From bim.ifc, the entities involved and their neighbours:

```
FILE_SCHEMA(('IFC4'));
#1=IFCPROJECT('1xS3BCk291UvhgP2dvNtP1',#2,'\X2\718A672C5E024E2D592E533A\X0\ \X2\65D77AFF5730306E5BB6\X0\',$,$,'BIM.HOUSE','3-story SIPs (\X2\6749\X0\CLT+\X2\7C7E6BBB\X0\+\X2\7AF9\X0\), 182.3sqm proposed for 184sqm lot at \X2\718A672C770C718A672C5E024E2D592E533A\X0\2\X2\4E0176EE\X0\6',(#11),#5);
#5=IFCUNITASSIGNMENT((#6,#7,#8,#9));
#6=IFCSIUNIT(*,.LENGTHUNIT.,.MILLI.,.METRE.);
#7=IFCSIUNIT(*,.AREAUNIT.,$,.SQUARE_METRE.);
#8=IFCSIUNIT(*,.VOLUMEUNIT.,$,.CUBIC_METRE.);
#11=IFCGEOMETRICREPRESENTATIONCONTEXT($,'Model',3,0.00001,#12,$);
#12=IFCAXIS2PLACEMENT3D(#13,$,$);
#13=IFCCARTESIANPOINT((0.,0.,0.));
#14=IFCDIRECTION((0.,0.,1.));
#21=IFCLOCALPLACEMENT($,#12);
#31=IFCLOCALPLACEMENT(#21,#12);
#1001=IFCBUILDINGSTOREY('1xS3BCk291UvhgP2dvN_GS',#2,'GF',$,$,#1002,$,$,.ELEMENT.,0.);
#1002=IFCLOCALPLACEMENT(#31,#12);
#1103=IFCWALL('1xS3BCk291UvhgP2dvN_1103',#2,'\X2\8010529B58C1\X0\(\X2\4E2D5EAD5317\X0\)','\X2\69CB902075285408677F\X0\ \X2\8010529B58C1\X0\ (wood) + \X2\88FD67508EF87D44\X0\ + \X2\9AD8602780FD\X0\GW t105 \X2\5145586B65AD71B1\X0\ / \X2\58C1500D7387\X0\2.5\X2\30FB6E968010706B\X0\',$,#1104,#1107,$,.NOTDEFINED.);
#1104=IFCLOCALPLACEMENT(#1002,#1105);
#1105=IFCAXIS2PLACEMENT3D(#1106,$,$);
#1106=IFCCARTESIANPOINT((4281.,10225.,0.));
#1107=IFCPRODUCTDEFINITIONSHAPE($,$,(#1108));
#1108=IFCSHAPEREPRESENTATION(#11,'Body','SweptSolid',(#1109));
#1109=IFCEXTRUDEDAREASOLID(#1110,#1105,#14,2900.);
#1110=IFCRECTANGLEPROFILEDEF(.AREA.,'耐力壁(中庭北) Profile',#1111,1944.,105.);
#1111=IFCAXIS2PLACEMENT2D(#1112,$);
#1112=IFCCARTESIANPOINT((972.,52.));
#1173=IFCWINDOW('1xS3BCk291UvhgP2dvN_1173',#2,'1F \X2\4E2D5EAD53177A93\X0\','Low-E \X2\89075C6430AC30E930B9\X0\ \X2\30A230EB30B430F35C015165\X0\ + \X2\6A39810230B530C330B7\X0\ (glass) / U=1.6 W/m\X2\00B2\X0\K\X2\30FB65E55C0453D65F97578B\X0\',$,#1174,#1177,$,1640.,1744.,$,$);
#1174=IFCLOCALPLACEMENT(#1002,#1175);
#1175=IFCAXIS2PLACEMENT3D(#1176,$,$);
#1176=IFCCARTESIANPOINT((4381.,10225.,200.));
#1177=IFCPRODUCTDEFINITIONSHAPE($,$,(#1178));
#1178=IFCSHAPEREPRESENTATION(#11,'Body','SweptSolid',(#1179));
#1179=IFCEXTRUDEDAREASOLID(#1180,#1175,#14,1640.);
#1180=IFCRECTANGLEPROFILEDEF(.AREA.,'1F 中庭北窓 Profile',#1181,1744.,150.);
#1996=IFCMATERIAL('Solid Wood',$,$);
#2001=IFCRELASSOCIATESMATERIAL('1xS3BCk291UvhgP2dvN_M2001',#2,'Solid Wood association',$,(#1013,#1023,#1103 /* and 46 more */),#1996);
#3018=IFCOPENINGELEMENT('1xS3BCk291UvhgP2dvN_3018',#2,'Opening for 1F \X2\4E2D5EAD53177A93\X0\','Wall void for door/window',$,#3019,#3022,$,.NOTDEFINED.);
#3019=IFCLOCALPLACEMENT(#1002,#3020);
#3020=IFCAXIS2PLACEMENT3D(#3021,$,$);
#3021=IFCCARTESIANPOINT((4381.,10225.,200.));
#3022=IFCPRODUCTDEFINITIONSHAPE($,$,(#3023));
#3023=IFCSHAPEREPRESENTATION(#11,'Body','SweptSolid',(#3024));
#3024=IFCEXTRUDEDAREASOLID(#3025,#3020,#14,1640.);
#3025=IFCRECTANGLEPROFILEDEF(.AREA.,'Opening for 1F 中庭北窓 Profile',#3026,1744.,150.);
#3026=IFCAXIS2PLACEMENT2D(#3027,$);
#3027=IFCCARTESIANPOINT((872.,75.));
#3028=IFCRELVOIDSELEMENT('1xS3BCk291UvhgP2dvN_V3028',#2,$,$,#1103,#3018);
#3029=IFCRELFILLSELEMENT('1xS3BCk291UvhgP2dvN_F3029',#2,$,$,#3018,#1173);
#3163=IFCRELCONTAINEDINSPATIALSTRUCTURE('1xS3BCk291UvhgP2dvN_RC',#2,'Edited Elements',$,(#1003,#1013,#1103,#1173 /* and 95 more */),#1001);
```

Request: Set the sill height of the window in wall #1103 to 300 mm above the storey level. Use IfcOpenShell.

```python
import numpy as np
import ifcopenshell
import ifcopenshell.api.geometry
import ifcopenshell.geom
import ifcopenshell.util.element
import ifcopenshell.util.placement
import ifcopenshell.util.shape
import ifcopenshell.util.unit

model = ifcopenshell.open("bim.ifc")
unit_scale = ifcopenshell.util.unit.calculate_unit_scale(model)

window = model.by_id(1173)
opening = window.FillsVoids[0].RelatingOpeningElement
storey = ifcopenshell.util.element.get_container(window, ifc_class="IfcBuildingStorey")
level = ifcopenshell.util.placement.get_local_placement(storey.ObjectPlacement)[2, 3]

# The opening's origin need not be at the sill, so measure its lowest point.
shape = ifcopenshell.geom.create_shape(ifcopenshell.geom.settings(), opening)
bottom = ifcopenshell.util.shape.get_shape_bottom_elevation(shape, shape.geometry) / unit_scale
dz = level + 0.3 / unit_scale - bottom

shift = np.array([0.0, 0.0, dz])
# The window is not placed relative to its opening, so move both.
for product in (opening, window):
    matrix = ifcopenshell.util.placement.get_local_placement(product.ObjectPlacement)
    matrix[:3, 3] += shift
    ifcopenshell.api.geometry.edit_object_placement(model, product=product, matrix=matrix, is_si=False)

print(f"moved by {dz * unit_scale:+.3f} m")

model.write("bim_v2.ifc")
```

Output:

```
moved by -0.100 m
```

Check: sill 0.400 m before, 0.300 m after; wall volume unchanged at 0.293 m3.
